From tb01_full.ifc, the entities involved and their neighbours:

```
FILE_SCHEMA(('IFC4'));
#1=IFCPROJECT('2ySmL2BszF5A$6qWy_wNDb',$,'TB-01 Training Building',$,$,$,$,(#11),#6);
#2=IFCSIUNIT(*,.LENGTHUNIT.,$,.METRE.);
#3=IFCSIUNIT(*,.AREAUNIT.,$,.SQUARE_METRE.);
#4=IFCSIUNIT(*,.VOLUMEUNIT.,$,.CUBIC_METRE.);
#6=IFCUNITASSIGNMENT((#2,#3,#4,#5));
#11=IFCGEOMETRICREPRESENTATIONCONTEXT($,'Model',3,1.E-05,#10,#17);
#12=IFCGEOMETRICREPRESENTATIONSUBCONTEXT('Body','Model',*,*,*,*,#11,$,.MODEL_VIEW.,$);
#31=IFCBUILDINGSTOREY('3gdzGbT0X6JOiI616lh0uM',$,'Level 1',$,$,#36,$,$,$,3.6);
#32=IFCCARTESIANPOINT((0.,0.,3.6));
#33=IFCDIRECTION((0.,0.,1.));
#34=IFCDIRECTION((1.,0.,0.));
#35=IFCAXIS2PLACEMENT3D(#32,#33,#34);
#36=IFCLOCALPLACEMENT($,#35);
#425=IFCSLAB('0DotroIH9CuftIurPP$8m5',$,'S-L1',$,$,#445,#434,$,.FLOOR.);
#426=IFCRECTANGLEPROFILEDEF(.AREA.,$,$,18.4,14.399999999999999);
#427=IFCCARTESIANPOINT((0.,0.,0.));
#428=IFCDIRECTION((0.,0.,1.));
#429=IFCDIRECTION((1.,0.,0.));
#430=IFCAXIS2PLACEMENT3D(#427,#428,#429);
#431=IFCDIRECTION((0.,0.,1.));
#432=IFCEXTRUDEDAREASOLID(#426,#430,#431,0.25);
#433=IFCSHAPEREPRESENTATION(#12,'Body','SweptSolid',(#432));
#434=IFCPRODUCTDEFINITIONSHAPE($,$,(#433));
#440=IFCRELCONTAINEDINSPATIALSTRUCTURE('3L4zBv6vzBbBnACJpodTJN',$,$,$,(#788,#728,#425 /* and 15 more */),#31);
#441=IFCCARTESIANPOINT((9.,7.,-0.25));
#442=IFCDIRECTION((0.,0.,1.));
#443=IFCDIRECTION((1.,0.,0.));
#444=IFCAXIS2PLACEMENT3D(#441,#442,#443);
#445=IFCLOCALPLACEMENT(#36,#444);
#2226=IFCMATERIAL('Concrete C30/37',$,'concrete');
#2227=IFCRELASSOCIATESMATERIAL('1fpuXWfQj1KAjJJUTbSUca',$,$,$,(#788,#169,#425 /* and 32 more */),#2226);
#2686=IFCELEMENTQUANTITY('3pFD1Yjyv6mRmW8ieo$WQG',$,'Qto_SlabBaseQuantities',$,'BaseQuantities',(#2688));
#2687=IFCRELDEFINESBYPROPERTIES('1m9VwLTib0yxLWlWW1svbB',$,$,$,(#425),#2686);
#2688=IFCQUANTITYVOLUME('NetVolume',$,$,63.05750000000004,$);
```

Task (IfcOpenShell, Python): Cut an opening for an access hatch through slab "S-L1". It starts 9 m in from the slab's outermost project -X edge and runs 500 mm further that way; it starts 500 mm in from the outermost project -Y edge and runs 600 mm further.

```python
import numpy as np
import ifcopenshell
import ifcopenshell.api.feature
import ifcopenshell.api.geometry
import ifcopenshell.api.pset
import ifcopenshell.api.root
import ifcopenshell.geom
import ifcopenshell.util.element
import ifcopenshell.util.placement
import ifcopenshell.util.representation
import ifcopenshell.util.shape
import ifcopenshell.util.unit

model = ifcopenshell.open("tb01_full.ifc")
unit_scale = ifcopenshell.util.unit.calculate_unit_scale(model)
volume_scale = ifcopenshell.util.unit.calculate_unit_scale(model, "VOLUMEUNIT")
settings = ifcopenshell.geom.settings()


def volume(element):
    """Net volume in cubic metres, openings subtracted."""
    shape = ifcopenshell.geom.create_shape(settings, element)
    return ifcopenshell.util.shape.get_volume(shape.geometry)


slab = model.by_guid("0DotroIH9CuftIurPP$8m5")
before = volume(slab)

# Extent in the slab's own axes, in metres. The edges named are its -X and -Y sides.
slab_shape = ifcopenshell.geom.create_shape(settings, slab)
vertices = ifcopenshell.util.shape.get_vertices(slab_shape.geometry)
x_min, y_min, bottom = vertices.min(axis=0)
top = vertices[:, 2].max()

opening = ifcopenshell.api.root.create_entity(model, ifc_class="IfcOpeningElement", name="Access hatch opening", predefined_type="OPENING")
context = ifcopenshell.util.representation.get_context(model, "Model", "Body", "MODEL_VIEW")
width, depth = 0.5, 0.6
outline = [(0.0, 0.0), (width, 0.0), (width, depth), (0.0, depth), (0.0, 0.0)]
# Overshoot both faces by 50 mm so the cut is clean.
shape = ifcopenshell.api.geometry.add_slab_representation(
    model, context=context, depth=top - bottom + 0.1, polyline=outline
)
ifcopenshell.api.geometry.assign_representation(model, product=opening, representation=shape)

matrix = ifcopenshell.util.placement.get_local_placement(slab.ObjectPlacement)
matrix[:, 3] = matrix @ np.append(np.array([x_min + 9, y_min + 0.5, bottom - 0.05]) / unit_scale, 1.0)
ifcopenshell.api.geometry.edit_object_placement(model, product=opening, matrix=matrix, is_si=False)
ifcopenshell.api.feature.add_feature(model, feature=opening, element=slab)

after = volume(slab)

# Update the slab's stored quantities.
qto = model.by_id(ifcopenshell.util.element.get_pset(slab, "Qto_SlabBaseQuantities", should_inherit=False)["id"])
ifcopenshell.api.pset.edit_qto(model, qto=qto, properties={"NetVolume": after / volume_scale})

print(f"slab volume {before:.3f} -> {after:.3f} m3")

model.write("tb01_full_v2.ifc")
```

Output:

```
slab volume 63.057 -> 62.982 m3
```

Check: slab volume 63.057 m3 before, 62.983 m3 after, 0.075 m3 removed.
